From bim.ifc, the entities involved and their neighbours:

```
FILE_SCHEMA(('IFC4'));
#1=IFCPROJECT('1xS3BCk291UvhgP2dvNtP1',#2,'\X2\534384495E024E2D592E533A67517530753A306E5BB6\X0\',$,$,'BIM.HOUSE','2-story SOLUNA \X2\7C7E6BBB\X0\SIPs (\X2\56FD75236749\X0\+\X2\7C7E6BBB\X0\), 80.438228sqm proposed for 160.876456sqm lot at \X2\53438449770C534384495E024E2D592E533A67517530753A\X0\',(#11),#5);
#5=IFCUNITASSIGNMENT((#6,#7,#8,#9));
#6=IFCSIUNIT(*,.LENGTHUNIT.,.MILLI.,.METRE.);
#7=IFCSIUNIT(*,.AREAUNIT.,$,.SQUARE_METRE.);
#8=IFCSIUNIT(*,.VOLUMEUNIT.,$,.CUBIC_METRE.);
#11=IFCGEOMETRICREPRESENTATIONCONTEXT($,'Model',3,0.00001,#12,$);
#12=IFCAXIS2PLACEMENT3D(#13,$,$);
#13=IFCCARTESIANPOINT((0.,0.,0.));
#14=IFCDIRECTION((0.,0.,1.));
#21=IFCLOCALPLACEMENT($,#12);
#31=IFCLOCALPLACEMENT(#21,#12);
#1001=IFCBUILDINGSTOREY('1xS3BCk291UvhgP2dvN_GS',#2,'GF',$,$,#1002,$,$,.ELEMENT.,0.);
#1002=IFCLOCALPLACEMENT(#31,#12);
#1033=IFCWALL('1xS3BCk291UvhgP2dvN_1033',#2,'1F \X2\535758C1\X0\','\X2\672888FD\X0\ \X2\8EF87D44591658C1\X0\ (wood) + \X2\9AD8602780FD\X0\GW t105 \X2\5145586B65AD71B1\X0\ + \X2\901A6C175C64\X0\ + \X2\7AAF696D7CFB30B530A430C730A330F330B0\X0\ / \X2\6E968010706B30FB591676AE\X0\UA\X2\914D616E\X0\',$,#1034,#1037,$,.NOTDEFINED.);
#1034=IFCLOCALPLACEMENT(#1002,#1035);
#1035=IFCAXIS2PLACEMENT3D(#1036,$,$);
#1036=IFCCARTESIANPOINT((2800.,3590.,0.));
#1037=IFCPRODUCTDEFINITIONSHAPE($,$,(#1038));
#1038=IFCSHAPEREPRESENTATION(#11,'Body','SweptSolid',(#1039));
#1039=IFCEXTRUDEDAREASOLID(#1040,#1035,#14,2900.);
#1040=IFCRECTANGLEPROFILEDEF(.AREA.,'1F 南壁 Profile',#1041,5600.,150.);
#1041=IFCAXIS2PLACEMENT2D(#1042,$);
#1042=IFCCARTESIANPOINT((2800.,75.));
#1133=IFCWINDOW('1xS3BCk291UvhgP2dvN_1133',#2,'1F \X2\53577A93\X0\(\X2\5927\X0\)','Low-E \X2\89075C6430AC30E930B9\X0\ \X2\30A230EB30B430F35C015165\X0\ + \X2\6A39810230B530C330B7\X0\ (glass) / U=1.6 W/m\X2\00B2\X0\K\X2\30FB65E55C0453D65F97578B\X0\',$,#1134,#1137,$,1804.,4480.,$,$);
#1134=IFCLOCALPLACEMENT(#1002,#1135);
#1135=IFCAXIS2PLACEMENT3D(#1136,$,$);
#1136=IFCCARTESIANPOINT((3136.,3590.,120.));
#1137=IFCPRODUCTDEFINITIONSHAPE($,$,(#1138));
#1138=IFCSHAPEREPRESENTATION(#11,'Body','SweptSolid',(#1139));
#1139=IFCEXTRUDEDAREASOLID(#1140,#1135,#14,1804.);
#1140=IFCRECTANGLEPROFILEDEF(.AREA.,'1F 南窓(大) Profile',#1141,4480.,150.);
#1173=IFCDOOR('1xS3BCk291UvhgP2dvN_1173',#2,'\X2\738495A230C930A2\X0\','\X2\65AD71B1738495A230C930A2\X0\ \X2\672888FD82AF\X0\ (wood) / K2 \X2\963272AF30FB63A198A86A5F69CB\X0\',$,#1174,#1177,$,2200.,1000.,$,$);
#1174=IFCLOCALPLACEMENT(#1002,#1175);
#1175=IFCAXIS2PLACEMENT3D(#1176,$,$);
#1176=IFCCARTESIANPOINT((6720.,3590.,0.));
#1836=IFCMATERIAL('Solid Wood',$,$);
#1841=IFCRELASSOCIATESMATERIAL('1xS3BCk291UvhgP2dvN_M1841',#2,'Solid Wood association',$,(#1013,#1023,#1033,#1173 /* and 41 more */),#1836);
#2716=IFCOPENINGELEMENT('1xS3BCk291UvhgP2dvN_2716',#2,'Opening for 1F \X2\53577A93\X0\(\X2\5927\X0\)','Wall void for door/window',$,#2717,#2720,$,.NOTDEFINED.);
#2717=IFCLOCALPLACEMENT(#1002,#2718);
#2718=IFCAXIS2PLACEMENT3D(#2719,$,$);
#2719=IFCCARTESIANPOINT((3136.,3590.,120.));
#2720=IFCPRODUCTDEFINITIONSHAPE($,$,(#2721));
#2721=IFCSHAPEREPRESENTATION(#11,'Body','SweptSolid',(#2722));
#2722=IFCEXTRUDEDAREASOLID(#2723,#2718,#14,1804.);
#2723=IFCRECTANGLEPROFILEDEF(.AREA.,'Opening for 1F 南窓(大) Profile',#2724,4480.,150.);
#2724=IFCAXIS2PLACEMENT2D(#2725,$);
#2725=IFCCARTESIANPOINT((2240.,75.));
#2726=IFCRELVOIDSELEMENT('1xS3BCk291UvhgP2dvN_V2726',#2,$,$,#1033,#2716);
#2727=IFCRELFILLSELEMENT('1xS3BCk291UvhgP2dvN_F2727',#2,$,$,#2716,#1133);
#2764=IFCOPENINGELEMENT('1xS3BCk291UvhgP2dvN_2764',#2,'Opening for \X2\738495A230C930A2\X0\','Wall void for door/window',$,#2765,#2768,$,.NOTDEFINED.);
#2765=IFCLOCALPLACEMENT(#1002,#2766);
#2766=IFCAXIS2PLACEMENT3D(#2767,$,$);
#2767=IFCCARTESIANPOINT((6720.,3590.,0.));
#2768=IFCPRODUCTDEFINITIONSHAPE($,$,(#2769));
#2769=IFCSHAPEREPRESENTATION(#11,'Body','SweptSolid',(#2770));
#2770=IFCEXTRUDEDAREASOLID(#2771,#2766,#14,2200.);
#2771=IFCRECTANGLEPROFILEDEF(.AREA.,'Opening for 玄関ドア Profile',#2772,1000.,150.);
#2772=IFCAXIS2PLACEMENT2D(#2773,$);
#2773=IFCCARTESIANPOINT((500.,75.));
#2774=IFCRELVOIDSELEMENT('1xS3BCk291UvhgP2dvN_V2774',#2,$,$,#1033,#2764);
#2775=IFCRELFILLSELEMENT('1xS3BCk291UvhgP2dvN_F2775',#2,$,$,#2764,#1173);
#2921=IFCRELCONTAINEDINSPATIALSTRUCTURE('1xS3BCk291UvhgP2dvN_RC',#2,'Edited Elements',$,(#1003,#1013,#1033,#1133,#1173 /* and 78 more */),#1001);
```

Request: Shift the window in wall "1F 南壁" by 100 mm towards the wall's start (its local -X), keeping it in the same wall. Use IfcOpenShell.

```python
import ifcopenshell
import ifcopenshell.api.geometry
import ifcopenshell.util.placement
import ifcopenshell.util.unit

model = ifcopenshell.open("bim.ifc")
unit_scale = ifcopenshell.util.unit.calculate_unit_scale(model)

window = model.by_id(1133)
opening = window.FillsVoids[0].RelatingOpeningElement
wall = opening.VoidsElements[0].RelatingBuildingElement

wall_matrix = ifcopenshell.util.placement.get_local_placement(wall.ObjectPlacement)
shift = wall_matrix[:3, 0] * -0.1 / unit_scale
before = ifcopenshell.util.placement.get_local_placement(window.ObjectPlacement)[:3, 3].copy()

# The window is not placed relative to its opening, so move both.
for product in (opening, window):
    matrix = ifcopenshell.util.placement.get_local_placement(product.ObjectPlacement)
    matrix[:3, 3] += shift
    ifcopenshell.api.geometry.edit_object_placement(model, product=product, matrix=matrix, is_si=False)

after = ifcopenshell.util.placement.get_local_placement(window.ObjectPlacement)[:3, 3]
print("window moved by", (after - before).round(3) + 0.0)

model.write("bim_rev.ifc")
```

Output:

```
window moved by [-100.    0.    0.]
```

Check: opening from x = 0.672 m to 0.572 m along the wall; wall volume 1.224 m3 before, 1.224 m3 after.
